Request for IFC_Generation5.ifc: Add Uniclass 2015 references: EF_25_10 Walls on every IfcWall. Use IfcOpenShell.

First a look at what the model holds.

```python
import ifcopenshell

model = ifcopenshell.open("IFC_Generation5.ifc")
print(model.schema)
print("classifications:", [c.Name for c in model.by_type("IfcClassification")])
for ifc_class in ("IfcDoor", "IfcRoof", "IfcStair", "IfcWall", "IfcWindow"):
    print(ifc_class, len(model.by_type(ifc_class)))
```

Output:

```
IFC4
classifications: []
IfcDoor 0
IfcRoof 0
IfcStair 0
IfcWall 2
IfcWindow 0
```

```python
import ifcopenshell
import ifcopenshell.api.classification

model = ifcopenshell.open("IFC_Generation5.ifc")

system = ifcopenshell.api.classification.add_classification(model, classification="Uniclass 2015")

codes = {
    "IfcWall": ("EF_25_10", "Walls"),
}
for ifc_class, (code, name) in codes.items():
    products = model.by_type(ifc_class)
    ifcopenshell.api.classification.add_reference(
        model, products=products, classification=system, identification=code, name=name
    )
    print(code, len(products))

model.write("IFC_Generation5_updated.ifc")
```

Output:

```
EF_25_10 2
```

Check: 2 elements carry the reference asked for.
